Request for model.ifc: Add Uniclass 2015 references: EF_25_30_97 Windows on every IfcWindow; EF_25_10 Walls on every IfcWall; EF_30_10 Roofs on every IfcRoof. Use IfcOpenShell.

First a look at what the model holds.

```python
import ifcopenshell

model = ifcopenshell.open("model.ifc")
print(model.schema)
print("classifications:", [c.Name for c in model.by_type("IfcClassification")])
for ifc_class in ("IfcDoor", "IfcRoof", "IfcStair", "IfcWall", "IfcWindow"):
    print(ifc_class, len(model.by_type(ifc_class)))
```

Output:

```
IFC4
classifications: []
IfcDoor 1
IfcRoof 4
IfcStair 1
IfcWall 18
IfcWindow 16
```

```python
import ifcopenshell
import ifcopenshell.api.classification

model = ifcopenshell.open("model.ifc")

system = ifcopenshell.api.classification.add_classification(model, classification="Uniclass 2015")

codes = {
    "IfcWindow": ("EF_25_30_97", "Windows"),
    "IfcWall": ("EF_25_10", "Walls"),
    "IfcRoof": ("EF_30_10", "Roofs"),
}
for ifc_class, (code, name) in codes.items():
    products = model.by_type(ifc_class)
    ifcopenshell.api.classification.add_reference(
        model, products=products, classification=system, identification=code, name=name
    )
    print(code, len(products))

model.write("model-out.ifc")
```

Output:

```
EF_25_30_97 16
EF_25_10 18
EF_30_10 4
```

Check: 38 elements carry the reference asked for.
